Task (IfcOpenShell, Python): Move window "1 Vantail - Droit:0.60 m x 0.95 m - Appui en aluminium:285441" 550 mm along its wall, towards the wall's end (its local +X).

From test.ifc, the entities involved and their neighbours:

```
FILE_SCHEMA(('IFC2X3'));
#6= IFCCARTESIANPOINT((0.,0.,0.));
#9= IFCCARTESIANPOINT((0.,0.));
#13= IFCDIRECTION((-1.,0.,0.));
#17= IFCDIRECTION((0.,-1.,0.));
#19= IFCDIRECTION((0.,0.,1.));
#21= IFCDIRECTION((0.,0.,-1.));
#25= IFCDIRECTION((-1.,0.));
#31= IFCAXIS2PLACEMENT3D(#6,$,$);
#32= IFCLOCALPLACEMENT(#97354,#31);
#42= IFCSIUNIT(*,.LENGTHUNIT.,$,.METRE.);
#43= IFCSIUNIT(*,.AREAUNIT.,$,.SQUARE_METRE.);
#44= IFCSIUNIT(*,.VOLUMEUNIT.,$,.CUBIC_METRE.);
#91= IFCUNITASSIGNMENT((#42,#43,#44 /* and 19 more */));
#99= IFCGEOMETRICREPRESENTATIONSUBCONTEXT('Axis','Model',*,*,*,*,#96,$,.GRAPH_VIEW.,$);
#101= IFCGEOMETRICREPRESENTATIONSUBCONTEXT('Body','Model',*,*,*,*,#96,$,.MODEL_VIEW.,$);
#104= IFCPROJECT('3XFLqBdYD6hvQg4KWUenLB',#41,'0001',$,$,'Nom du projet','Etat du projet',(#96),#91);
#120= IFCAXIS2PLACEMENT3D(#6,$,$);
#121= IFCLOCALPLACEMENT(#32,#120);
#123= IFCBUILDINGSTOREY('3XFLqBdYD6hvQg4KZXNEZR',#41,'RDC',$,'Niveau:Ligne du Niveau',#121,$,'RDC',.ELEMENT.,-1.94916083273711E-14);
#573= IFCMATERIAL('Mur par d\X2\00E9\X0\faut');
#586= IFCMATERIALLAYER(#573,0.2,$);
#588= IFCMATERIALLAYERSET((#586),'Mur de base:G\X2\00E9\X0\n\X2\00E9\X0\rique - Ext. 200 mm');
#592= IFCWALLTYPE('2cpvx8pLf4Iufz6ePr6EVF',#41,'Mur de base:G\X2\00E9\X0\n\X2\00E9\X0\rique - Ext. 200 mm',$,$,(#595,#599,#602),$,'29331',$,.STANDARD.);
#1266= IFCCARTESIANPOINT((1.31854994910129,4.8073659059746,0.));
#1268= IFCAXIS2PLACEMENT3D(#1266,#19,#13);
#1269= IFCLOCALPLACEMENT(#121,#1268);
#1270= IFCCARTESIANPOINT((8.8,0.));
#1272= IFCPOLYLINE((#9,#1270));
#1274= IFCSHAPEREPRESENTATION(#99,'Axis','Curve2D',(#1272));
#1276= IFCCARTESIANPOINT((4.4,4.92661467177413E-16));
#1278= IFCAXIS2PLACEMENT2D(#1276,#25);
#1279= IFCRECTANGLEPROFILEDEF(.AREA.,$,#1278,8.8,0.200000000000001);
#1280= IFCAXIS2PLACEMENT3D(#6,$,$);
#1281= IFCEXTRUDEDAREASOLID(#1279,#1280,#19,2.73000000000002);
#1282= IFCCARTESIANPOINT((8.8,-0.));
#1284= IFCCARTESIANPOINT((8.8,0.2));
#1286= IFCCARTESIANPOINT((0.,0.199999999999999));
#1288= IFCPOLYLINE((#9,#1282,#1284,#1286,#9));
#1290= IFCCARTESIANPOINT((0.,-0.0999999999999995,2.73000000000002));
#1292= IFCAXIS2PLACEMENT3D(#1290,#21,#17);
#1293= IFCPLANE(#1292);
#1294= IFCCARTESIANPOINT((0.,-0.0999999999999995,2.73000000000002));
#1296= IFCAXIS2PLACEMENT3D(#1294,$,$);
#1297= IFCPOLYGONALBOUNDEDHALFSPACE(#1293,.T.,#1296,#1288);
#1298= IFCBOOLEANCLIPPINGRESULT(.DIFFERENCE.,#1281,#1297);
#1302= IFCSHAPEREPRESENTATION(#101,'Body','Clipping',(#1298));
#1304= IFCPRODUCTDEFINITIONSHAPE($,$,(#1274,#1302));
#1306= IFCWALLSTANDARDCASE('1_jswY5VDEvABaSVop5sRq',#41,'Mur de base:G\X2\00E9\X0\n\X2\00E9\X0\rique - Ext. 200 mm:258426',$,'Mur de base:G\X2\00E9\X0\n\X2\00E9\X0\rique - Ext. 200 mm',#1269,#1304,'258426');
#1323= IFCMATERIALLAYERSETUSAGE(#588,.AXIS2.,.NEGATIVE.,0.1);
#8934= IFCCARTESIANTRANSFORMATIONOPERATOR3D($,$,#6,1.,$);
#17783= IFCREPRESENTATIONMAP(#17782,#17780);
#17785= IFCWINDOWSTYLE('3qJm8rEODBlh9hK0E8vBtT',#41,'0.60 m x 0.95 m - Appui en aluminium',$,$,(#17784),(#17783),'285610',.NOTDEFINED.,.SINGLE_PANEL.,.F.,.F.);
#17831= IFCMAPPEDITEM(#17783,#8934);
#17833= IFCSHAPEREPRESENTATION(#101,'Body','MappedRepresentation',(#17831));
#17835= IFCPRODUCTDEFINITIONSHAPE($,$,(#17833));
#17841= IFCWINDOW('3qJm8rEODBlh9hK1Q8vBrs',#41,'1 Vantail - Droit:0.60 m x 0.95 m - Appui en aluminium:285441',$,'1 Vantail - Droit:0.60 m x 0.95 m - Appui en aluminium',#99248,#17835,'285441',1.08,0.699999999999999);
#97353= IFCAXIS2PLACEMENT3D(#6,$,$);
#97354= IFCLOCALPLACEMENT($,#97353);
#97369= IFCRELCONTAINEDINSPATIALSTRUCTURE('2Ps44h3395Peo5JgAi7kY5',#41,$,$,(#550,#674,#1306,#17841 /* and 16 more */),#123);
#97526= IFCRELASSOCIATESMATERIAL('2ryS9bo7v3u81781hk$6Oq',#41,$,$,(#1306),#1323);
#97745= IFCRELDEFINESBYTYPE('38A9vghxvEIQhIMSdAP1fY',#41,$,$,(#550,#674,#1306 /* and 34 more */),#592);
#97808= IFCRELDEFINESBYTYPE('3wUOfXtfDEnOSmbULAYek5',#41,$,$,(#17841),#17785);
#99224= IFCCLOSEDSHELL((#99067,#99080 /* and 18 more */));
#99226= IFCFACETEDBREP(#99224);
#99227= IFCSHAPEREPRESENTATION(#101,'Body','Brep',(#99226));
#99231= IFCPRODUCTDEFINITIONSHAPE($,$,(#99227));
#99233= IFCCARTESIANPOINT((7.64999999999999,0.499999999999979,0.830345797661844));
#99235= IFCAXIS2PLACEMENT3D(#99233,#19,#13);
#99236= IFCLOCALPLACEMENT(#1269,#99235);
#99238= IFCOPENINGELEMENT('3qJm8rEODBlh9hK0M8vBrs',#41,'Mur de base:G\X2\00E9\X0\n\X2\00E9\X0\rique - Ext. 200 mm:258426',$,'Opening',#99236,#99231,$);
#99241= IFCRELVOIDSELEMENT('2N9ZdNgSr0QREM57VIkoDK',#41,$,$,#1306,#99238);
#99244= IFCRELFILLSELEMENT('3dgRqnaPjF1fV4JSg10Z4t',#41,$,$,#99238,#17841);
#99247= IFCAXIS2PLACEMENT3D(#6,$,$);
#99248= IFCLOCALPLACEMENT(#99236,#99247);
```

```python
import ifcopenshell
import ifcopenshell.api.geometry
import ifcopenshell.util.placement
import ifcopenshell.util.unit

model = ifcopenshell.open("test.ifc")
unit_scale = ifcopenshell.util.unit.calculate_unit_scale(model)

window = model.by_guid("3qJm8rEODBlh9hK1Q8vBrs")
opening = window.FillsVoids[0].RelatingOpeningElement
wall = opening.VoidsElements[0].RelatingBuildingElement

wall_matrix = ifcopenshell.util.placement.get_local_placement(wall.ObjectPlacement)
shift = wall_matrix[:3, 0] * 0.55 / unit_scale
before = ifcopenshell.util.placement.get_local_placement(window.ObjectPlacement)[:3, 3].copy()

# The window is placed relative to its opening, so it follows when the opening moves.
matrix = ifcopenshell.util.placement.get_local_placement(opening.ObjectPlacement)
matrix[:3, 3] += shift
ifcopenshell.api.geometry.edit_object_placement(
    model, product=opening, matrix=matrix, is_si=False, should_transform_children=True
)

after = ifcopenshell.util.placement.get_local_placement(window.ObjectPlacement)[:3, 3]
print("window moved by", (after - before).round(3) + 0.0)

model.write("test-out.ifc")
```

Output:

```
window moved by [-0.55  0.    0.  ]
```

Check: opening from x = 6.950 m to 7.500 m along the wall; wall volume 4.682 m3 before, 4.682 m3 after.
